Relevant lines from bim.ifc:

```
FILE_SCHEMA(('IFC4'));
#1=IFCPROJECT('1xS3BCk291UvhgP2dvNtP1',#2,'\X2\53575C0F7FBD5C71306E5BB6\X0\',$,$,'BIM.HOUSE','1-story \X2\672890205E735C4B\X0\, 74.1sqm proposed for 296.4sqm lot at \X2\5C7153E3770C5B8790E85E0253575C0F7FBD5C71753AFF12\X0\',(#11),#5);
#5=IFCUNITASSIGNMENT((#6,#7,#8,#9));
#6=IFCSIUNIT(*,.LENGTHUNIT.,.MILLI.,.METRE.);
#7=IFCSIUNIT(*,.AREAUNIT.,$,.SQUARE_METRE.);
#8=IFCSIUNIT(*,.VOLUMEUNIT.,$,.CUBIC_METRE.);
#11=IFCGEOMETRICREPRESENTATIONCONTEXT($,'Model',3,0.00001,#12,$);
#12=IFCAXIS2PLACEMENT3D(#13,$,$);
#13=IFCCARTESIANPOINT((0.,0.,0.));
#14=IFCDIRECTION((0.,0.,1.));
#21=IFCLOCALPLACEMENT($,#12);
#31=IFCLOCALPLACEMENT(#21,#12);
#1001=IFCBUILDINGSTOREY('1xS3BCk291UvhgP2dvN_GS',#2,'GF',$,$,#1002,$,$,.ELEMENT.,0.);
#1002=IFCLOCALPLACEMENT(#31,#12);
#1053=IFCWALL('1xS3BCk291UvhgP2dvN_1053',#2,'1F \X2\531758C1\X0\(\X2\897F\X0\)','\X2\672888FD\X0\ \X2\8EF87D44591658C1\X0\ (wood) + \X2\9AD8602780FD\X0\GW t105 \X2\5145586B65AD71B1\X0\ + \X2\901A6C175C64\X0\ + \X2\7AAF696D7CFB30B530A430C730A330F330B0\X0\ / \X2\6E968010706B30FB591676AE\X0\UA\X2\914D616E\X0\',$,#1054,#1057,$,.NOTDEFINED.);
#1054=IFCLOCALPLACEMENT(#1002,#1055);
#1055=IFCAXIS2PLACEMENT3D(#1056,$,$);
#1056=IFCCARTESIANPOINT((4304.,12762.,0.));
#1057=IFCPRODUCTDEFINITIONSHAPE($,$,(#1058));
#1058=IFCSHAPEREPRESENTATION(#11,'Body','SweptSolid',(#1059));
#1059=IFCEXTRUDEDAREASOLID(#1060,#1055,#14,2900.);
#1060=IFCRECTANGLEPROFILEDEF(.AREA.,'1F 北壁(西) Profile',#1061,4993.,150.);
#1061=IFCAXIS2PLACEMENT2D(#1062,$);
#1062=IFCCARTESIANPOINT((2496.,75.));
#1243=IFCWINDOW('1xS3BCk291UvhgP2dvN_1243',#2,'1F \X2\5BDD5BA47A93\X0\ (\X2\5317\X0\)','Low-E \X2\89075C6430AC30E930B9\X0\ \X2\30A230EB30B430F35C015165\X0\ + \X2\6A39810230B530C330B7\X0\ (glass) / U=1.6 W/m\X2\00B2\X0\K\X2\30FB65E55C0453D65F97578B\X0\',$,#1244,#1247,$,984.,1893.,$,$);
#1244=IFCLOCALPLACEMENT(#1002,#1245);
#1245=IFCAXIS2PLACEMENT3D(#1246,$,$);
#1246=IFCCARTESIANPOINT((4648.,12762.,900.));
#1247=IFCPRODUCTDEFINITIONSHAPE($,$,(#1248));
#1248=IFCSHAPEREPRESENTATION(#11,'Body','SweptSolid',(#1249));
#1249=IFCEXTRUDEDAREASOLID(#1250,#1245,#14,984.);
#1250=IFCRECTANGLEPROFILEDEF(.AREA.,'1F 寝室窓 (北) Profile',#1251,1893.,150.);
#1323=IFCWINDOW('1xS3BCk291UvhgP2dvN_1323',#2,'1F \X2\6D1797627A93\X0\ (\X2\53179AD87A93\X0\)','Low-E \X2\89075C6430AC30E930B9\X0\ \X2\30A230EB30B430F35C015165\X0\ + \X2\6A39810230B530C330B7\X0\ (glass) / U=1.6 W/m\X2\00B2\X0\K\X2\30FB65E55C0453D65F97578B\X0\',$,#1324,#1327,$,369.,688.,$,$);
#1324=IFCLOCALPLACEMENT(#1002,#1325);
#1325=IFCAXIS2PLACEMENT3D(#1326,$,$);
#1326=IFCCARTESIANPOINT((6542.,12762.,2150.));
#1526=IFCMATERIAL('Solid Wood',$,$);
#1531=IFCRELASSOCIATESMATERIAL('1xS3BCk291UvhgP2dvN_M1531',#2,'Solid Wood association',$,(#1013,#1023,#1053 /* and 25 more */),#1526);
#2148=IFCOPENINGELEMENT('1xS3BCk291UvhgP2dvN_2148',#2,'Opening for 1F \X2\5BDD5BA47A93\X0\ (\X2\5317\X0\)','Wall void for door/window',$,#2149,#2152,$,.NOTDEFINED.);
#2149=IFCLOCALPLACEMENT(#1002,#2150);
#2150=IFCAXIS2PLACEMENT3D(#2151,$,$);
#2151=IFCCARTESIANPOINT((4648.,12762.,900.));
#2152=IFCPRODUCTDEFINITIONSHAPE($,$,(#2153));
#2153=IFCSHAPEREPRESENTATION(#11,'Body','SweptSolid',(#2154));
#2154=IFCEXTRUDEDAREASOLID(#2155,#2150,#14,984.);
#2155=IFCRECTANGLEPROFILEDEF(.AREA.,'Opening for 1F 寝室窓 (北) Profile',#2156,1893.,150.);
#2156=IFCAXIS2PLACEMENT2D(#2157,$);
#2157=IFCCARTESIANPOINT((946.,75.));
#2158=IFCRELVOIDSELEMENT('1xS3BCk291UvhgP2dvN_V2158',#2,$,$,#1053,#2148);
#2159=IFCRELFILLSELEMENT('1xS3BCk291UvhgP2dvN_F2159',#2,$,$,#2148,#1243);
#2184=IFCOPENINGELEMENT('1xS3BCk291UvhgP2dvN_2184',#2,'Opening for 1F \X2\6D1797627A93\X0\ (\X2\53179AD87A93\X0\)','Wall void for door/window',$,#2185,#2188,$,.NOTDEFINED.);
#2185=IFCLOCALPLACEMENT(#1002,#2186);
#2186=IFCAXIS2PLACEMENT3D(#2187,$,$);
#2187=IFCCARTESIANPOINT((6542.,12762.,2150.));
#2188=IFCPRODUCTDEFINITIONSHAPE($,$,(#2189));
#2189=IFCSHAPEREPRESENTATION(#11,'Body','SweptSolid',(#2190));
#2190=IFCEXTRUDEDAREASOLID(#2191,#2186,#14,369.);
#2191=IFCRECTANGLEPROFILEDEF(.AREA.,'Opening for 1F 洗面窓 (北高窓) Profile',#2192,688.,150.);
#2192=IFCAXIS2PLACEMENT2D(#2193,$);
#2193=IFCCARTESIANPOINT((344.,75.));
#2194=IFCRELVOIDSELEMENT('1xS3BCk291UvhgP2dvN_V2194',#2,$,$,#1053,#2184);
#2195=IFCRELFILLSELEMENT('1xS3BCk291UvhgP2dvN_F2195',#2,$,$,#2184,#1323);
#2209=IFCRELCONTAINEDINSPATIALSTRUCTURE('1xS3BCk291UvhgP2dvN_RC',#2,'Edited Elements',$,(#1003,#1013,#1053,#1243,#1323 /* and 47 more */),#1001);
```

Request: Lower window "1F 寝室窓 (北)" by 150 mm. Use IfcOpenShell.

```python
import numpy as np
import ifcopenshell
import ifcopenshell.api.geometry
import ifcopenshell.util.placement
import ifcopenshell.util.unit

model = ifcopenshell.open("bim.ifc")
unit_scale = ifcopenshell.util.unit.calculate_unit_scale(model)

window = model.by_id(1243)
opening = window.FillsVoids[0].RelatingOpeningElement
dz = -0.15 / unit_scale

shift = np.array([0.0, 0.0, dz])
# The window is not placed relative to its opening, so move both.
for product in (opening, window):
    matrix = ifcopenshell.util.placement.get_local_placement(product.ObjectPlacement)
    matrix[:3, 3] += shift
    ifcopenshell.api.geometry.edit_object_placement(model, product=product, matrix=matrix, is_si=False)

print(f"moved by {dz * unit_scale:+.3f} m")

model.write("bim_updated.ifc")
```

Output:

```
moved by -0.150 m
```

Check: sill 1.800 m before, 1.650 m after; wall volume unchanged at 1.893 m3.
